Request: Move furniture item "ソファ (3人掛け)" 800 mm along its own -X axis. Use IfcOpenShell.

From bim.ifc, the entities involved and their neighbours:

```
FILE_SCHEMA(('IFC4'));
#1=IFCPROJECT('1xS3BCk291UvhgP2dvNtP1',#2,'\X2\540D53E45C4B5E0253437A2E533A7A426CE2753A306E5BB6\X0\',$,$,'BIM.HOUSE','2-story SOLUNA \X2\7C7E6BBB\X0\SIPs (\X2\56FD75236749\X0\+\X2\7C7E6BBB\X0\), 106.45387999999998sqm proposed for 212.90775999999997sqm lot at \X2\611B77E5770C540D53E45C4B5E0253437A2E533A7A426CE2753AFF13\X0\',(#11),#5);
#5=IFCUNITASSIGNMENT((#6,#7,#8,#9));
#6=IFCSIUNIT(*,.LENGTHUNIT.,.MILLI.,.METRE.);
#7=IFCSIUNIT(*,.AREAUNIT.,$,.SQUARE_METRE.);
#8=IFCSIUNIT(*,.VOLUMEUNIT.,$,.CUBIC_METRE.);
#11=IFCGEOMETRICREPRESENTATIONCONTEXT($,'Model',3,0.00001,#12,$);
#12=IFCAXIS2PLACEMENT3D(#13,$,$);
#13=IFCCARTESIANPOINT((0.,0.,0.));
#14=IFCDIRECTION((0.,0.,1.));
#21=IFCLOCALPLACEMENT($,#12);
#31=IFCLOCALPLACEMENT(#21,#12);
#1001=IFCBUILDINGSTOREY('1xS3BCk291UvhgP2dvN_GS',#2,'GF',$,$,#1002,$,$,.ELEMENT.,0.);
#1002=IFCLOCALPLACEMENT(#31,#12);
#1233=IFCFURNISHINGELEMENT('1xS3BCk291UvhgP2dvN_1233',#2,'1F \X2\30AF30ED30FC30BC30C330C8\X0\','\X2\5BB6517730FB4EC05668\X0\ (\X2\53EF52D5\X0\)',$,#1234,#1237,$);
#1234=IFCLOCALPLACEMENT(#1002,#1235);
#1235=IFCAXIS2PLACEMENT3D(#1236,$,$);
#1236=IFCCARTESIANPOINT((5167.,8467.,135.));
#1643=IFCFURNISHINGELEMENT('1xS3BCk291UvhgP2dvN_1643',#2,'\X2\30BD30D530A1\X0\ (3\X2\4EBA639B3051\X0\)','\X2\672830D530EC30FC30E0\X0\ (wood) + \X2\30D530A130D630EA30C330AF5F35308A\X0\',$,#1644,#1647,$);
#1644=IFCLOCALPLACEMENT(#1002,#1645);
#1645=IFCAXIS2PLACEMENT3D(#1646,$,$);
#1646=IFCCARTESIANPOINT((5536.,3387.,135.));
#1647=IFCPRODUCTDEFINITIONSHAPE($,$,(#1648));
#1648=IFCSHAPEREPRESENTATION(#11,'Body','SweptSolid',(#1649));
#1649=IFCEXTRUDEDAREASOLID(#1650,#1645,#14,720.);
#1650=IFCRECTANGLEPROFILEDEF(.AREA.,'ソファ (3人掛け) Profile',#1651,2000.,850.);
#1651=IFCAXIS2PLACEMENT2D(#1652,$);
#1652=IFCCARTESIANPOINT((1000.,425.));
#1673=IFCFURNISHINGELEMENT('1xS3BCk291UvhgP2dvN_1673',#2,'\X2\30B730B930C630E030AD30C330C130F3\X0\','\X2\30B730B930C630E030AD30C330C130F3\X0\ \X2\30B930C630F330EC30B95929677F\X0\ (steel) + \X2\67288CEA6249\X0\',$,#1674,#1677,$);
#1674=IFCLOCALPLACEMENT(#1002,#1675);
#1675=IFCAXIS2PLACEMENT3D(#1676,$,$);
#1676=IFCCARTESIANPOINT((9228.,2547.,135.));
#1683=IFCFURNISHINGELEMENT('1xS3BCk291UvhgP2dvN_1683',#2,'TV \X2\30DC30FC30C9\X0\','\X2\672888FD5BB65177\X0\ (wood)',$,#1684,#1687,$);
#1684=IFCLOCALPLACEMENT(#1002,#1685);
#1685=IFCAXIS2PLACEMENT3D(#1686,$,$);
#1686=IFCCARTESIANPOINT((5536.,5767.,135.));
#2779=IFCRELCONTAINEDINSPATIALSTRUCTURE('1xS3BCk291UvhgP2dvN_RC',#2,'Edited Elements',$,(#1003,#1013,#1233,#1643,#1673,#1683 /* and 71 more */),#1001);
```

```python
import ifcopenshell
import ifcopenshell.api.geometry
import ifcopenshell.util.placement

model = ifcopenshell.open("bim.ifc")

item = model.by_guid("1xS3BCk291UvhgP2dvN_1643")
matrix = ifcopenshell.util.placement.get_local_placement(item.ObjectPlacement)
matrix[:3, 3] -= matrix[:3, 0] * 800.0
ifcopenshell.api.geometry.edit_object_placement(model, product=item, matrix=matrix, is_si=False)

print(ifcopenshell.util.placement.get_local_placement(item.ObjectPlacement).round(3) + 0.0)

model.write("bim_rev.ifc")
```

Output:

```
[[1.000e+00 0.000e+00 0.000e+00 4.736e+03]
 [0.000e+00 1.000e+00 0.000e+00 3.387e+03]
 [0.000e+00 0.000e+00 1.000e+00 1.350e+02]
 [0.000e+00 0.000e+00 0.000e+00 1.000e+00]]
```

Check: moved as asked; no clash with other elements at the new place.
